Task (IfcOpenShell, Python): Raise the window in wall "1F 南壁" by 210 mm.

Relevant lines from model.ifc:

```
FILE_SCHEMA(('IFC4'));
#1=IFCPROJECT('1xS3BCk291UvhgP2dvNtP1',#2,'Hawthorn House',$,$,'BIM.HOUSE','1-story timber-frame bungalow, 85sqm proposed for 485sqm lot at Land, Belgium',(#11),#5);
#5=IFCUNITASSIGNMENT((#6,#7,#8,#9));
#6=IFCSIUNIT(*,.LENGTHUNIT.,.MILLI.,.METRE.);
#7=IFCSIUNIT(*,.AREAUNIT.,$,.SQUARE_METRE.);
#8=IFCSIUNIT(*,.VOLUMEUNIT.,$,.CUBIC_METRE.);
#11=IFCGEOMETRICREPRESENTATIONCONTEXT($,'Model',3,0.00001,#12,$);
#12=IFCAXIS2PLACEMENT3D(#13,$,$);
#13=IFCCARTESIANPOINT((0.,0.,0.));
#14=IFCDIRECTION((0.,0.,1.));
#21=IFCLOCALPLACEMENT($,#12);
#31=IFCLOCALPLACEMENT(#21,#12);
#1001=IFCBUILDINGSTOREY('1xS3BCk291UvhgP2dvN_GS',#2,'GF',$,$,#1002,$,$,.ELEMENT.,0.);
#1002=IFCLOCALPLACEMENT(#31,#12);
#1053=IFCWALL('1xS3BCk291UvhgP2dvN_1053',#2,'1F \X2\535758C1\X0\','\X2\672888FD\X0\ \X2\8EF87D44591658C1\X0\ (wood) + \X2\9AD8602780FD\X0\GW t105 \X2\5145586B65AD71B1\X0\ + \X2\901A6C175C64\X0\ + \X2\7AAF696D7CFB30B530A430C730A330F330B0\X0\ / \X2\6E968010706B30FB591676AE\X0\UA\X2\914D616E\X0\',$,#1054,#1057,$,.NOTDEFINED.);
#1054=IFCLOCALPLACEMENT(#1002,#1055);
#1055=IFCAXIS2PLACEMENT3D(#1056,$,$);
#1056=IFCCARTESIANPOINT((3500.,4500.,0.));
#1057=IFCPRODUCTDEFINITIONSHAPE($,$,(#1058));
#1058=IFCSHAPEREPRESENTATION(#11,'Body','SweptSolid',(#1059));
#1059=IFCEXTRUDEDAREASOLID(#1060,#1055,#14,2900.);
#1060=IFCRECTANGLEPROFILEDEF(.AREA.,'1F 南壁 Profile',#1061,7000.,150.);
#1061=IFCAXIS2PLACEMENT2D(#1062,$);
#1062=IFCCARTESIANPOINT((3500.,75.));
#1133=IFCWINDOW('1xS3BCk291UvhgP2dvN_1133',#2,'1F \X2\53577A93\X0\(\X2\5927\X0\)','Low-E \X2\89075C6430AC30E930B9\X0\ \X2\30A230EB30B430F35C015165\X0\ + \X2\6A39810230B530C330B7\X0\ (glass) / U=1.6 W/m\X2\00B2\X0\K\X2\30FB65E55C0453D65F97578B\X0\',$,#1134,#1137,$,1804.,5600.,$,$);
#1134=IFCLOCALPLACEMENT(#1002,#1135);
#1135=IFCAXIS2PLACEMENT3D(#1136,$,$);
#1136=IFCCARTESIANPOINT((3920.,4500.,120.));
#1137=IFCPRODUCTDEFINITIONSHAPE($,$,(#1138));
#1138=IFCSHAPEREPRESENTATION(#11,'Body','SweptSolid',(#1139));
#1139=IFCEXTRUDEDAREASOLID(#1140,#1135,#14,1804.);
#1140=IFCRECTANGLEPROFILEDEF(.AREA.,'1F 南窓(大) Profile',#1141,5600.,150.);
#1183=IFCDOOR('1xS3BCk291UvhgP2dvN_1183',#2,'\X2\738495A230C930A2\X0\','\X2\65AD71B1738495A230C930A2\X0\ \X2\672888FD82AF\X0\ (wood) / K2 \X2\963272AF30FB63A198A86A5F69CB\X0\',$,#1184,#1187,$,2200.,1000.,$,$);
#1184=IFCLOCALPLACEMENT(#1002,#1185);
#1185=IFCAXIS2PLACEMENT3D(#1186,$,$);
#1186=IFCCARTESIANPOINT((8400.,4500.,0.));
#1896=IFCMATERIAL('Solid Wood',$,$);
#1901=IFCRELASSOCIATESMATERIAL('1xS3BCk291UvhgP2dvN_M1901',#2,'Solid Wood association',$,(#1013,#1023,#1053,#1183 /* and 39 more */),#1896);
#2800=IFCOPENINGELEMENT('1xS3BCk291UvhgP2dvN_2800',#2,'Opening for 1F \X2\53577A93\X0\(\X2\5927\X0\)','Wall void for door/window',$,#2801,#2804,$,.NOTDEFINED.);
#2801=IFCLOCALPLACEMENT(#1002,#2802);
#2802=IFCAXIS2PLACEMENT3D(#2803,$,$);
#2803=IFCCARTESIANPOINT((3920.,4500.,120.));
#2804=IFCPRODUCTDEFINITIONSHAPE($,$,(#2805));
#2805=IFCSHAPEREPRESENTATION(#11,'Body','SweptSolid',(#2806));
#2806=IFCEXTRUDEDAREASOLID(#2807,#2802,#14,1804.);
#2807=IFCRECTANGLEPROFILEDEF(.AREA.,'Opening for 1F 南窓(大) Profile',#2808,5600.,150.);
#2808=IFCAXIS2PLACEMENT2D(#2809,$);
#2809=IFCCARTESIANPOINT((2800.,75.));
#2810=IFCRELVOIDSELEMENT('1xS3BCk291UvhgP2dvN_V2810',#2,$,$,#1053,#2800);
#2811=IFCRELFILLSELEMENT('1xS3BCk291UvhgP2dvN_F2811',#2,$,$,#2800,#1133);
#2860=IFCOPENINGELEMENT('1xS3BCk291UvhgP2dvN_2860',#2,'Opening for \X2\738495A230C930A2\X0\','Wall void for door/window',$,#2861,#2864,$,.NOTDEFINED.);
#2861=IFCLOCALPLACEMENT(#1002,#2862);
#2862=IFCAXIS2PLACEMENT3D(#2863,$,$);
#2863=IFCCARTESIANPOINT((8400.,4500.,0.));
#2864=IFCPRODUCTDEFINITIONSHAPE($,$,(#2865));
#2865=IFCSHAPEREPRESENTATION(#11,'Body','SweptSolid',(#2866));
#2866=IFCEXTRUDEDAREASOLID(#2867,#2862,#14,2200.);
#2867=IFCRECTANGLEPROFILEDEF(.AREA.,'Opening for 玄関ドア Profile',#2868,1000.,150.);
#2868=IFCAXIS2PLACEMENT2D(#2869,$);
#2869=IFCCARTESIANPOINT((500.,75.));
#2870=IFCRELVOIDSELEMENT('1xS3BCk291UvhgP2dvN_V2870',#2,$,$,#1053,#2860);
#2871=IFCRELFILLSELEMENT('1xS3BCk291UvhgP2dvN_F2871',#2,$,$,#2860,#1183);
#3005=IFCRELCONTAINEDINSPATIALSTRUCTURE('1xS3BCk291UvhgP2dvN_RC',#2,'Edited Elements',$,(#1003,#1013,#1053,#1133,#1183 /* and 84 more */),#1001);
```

```python
import numpy as np
import ifcopenshell
import ifcopenshell.api.geometry
import ifcopenshell.util.placement
import ifcopenshell.util.unit

model = ifcopenshell.open("model.ifc")
unit_scale = ifcopenshell.util.unit.calculate_unit_scale(model)

window = model.by_guid("1xS3BCk291UvhgP2dvN_1133")
opening = window.FillsVoids[0].RelatingOpeningElement
dz = 0.21 / unit_scale

shift = np.array([0.0, 0.0, dz])
# The window is not placed relative to its opening, so move both.
for product in (opening, window):
    matrix = ifcopenshell.util.placement.get_local_placement(product.ObjectPlacement)
    matrix[:3, 3] += shift
    ifcopenshell.api.geometry.edit_object_placement(model, product=product, matrix=matrix, is_si=False)

print(f"moved by {dz * unit_scale:+.3f} m")

model.write("model-out.ifc")
```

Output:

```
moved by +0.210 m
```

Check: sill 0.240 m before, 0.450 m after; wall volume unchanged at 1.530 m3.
